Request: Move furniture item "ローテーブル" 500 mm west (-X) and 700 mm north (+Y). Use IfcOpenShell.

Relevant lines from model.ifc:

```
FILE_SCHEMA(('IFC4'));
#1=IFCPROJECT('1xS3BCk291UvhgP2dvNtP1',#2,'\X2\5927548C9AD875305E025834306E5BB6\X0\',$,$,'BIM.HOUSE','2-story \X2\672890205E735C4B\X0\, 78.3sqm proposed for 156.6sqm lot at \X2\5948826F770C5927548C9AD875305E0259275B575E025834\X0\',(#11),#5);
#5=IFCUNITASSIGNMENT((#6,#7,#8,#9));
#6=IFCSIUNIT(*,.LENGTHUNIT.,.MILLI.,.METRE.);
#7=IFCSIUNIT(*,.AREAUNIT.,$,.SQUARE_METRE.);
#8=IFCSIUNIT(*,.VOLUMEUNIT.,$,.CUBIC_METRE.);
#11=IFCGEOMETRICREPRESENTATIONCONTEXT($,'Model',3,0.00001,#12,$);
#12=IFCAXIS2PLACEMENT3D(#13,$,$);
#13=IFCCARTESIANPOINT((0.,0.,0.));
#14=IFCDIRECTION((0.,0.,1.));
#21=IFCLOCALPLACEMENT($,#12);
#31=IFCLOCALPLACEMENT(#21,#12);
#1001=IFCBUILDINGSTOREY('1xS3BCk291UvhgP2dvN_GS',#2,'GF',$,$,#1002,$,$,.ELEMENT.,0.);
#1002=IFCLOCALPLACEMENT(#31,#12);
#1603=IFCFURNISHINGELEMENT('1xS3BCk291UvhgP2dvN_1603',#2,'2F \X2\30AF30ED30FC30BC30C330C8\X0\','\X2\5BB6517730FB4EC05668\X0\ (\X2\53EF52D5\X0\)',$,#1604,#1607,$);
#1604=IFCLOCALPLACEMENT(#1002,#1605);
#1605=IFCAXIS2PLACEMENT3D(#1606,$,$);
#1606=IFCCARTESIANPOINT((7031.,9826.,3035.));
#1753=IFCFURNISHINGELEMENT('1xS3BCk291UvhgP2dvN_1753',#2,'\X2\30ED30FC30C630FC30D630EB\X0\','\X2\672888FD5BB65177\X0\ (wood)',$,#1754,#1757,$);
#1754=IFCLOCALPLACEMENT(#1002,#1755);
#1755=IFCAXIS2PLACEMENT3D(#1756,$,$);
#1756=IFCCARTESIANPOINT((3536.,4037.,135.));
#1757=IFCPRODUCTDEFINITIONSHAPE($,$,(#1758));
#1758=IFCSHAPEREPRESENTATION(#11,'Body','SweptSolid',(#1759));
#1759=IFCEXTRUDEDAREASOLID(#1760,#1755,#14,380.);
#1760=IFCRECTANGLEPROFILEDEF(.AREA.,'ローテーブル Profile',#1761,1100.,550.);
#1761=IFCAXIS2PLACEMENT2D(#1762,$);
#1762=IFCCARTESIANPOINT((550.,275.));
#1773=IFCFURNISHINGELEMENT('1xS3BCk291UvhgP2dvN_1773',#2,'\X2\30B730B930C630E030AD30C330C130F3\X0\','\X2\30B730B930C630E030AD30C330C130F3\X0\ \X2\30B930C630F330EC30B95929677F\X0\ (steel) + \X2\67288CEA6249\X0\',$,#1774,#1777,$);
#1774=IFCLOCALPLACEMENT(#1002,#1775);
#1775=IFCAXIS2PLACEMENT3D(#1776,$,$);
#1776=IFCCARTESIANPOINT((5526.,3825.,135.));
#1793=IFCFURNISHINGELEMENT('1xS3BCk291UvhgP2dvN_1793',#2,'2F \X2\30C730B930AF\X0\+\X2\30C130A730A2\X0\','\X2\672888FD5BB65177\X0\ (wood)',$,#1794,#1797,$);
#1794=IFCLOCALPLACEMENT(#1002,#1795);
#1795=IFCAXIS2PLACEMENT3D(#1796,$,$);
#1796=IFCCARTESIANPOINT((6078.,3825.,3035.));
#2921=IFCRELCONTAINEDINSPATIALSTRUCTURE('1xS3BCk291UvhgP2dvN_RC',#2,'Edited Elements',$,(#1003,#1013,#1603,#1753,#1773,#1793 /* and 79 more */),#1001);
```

```python
import ifcopenshell
import ifcopenshell.api.geometry
import ifcopenshell.util.placement

model = ifcopenshell.open("model.ifc")

item = model.by_guid("1xS3BCk291UvhgP2dvN_1753")
matrix = ifcopenshell.util.placement.get_local_placement(item.ObjectPlacement)
matrix[0, 3] -= 500.0
matrix[1, 3] += 700.0
ifcopenshell.api.geometry.edit_object_placement(model, product=item, matrix=matrix, is_si=False)

print(ifcopenshell.util.placement.get_local_placement(item.ObjectPlacement).round(3) + 0.0)

model.write("model_edited.ifc")
```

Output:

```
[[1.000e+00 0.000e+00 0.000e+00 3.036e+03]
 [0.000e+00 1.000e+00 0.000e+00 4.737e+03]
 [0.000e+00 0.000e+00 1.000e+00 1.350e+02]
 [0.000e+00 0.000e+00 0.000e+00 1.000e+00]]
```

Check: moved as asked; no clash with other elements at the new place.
